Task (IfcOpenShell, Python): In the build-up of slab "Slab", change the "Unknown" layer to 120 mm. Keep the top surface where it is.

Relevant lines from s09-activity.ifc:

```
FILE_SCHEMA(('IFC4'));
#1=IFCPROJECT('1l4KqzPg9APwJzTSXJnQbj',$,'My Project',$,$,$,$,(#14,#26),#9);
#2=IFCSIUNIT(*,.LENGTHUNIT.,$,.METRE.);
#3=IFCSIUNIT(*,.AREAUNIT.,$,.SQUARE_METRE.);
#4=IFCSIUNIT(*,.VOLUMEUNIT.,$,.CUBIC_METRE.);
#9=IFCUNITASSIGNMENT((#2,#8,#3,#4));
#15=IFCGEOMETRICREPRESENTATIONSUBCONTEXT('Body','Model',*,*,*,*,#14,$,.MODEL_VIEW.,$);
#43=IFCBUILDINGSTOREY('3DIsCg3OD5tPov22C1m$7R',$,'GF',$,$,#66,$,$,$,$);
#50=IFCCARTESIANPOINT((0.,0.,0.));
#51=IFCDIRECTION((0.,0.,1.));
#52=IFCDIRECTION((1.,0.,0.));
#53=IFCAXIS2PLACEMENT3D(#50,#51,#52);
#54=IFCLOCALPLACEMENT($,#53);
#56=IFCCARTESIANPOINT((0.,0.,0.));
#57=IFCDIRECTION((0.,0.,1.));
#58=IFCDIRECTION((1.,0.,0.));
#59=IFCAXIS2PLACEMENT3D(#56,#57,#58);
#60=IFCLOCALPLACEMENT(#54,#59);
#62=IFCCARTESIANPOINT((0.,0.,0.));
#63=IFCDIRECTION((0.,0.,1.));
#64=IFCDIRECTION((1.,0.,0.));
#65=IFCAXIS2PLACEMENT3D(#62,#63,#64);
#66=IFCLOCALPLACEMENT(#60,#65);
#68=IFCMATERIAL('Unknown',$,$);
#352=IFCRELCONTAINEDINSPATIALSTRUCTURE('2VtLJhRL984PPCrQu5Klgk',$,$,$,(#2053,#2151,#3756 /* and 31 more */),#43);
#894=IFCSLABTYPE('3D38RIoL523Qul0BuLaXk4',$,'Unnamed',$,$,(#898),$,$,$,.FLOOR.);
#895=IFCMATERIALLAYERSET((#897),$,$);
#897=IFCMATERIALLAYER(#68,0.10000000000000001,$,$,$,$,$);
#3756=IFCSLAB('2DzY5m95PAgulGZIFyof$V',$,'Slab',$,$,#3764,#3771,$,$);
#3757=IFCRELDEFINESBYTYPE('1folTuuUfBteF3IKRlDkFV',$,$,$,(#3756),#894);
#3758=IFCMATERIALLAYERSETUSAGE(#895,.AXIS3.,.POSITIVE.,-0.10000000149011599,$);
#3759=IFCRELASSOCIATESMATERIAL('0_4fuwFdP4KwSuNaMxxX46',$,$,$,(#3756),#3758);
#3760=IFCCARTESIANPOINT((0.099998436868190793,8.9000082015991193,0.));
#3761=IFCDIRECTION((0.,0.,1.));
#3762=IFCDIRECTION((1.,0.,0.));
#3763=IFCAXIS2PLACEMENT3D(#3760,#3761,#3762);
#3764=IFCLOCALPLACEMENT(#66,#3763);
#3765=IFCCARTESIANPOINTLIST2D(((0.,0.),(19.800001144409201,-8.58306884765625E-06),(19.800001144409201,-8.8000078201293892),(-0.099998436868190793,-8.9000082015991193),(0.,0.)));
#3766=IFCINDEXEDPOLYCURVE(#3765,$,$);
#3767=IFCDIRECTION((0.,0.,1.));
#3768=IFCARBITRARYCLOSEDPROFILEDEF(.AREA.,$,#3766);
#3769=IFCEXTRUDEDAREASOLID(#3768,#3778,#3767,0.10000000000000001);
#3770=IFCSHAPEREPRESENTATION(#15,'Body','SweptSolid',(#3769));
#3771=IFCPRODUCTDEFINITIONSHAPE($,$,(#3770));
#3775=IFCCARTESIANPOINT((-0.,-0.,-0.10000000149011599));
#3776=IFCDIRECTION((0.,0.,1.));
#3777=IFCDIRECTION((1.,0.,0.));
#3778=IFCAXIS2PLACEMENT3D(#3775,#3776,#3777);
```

```python
import ifcopenshell
import ifcopenshell.util.element
import ifcopenshell.util.representation
import ifcopenshell.util.unit

model = ifcopenshell.open("s09-activity.ifc")
unit_scale = ifcopenshell.util.unit.calculate_unit_scale(model)

layer_set = model.by_id(895)
layer = next(l for l in layer_set.MaterialLayers if l.Material and l.Material.Name == "Unknown")
change = 0.12 / unit_scale - layer.LayerThickness
layer.LayerThickness += change

# Geometry does not follow the layer set by itself.
slabs = [e for e in ifcopenshell.util.element.get_elements_by_material(model, layer_set) if e.is_a("IfcSlab")]
for slab in sorted(slabs, key=lambda e: e.id()):
    body = ifcopenshell.util.representation.get_representation(slab, "Model", "Body")
    solid = body.Items[0]
    old_depth = solid.Depth
    solid.Depth += change
    # Extruded upwards: lower the start of the extrusion so the top stays.
    x, y, z = solid.Position.Location.Coordinates
    solid.Position.Location = model.createIfcCartesianPoint((x, y, z - change))
    print(slab.id(), f"{old_depth:g} -> {solid.Depth:g}")

# The layers are counted up from the underside, which has moved.
for usage in {ifcopenshell.util.element.get_material(slab) for slab in slabs}:
    usage.OffsetFromReferenceLine -= change

model.write("s09-activity_rev.ifc")
```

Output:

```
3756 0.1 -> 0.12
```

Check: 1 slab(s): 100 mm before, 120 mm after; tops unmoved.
